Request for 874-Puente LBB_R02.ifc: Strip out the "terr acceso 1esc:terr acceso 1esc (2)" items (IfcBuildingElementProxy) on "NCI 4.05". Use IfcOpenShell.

First a look at what the model holds.

```python
import ifcopenshell
import ifcopenshell.util.element

model = ifcopenshell.open("874-Puente LBB_R02.ifc")
print(model.schema)
storey = next(s for s in model.by_type("IfcBuildingStorey") if s.Name == "NCI 4.05")
proxies = [e for e in ifcopenshell.util.element.get_decomposition(storey) if e.is_a("IfcBuildingElementProxy")]
seen = {}
for e in proxies:
    element_type = ifcopenshell.util.element.get_type(e)
    name = element_type.Name if element_type not in (None, e) else None
    seen[name] = seen.get(name, 0) + 1
for name, count in sorted(seen.items(), key=str):
    print(count, "x", name)
```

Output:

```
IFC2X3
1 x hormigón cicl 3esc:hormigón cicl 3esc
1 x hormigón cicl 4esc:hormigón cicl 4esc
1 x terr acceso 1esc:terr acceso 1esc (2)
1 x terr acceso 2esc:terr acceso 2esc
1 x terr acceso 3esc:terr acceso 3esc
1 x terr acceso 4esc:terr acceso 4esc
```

```python
import ifcopenshell
import ifcopenshell.api.root
import ifcopenshell.util.element

model = ifcopenshell.open("874-Puente LBB_R02.ifc")

storey = next(s for s in model.by_type("IfcBuildingStorey") if s.Name == "NCI 4.05")
proxies = [e for e in ifcopenshell.util.element.get_decomposition(storey) if e.is_a("IfcBuildingElementProxy")]
targets = [e for e in proxies if (t := ifcopenshell.util.element.get_type(e)) not in (None, e) and t.Name == "terr acceso 1esc:terr acceso 1esc (2)"]

for e in targets:
    ifcopenshell.api.root.remove_product(model, product=e)
print(len(targets), "removed")

model.write("874-Puente LBB_R02_edited.ifc")
```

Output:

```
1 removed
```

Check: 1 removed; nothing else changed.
